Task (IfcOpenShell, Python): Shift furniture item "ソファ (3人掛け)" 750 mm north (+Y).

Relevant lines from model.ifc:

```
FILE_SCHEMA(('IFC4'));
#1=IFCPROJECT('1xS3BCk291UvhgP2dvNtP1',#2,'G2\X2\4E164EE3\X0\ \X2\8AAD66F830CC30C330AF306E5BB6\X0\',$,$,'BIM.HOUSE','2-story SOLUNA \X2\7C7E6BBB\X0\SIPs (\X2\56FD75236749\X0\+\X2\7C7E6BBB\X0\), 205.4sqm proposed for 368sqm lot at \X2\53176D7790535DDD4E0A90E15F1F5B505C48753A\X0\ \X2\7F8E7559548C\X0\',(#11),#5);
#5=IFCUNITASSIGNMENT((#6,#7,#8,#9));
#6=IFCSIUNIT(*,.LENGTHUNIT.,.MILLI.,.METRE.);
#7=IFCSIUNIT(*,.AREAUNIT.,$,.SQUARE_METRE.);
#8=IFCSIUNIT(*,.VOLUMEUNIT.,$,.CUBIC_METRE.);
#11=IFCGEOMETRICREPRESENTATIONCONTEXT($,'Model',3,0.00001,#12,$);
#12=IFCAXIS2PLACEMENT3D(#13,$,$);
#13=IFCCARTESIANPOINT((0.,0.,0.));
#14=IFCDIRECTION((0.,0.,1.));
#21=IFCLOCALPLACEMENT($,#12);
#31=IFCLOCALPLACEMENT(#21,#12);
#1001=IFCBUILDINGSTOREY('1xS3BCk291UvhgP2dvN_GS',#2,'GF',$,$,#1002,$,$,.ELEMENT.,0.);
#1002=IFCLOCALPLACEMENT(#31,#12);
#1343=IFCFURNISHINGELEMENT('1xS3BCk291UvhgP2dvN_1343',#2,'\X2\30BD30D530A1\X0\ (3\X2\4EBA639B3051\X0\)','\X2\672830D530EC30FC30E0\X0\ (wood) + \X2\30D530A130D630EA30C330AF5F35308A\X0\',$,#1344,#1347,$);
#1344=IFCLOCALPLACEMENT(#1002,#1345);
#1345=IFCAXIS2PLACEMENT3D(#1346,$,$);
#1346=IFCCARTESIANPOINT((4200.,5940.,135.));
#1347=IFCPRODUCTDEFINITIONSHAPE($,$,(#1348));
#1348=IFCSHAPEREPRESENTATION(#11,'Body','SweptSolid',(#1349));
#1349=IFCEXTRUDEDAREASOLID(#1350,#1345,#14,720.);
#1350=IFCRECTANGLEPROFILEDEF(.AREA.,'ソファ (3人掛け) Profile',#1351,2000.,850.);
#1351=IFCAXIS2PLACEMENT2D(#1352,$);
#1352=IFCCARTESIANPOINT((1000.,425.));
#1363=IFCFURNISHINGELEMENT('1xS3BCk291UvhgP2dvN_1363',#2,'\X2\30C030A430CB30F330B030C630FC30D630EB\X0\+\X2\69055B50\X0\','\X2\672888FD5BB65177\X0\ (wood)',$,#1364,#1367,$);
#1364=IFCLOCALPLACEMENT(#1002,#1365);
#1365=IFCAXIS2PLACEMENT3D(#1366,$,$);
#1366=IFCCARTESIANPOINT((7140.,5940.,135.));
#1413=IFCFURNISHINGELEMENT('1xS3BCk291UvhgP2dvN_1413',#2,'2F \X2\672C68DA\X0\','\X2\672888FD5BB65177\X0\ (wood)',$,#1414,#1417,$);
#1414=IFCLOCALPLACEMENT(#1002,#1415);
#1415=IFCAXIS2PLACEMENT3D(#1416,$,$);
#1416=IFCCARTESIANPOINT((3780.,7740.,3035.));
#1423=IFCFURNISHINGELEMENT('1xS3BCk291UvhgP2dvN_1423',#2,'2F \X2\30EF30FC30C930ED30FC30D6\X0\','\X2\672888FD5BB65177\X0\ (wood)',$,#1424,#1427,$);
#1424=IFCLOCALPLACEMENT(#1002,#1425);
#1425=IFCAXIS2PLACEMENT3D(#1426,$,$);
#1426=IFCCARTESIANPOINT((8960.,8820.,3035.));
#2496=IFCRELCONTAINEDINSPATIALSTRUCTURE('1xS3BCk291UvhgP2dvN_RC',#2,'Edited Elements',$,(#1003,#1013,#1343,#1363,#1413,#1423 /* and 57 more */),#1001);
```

```python
import ifcopenshell
import ifcopenshell.api.geometry
import ifcopenshell.util.placement

model = ifcopenshell.open("model.ifc")

item = model.by_guid("1xS3BCk291UvhgP2dvN_1343")
matrix = ifcopenshell.util.placement.get_local_placement(item.ObjectPlacement)
matrix[1, 3] += 750.0
ifcopenshell.api.geometry.edit_object_placement(model, product=item, matrix=matrix, is_si=False)

print(ifcopenshell.util.placement.get_local_placement(item.ObjectPlacement).round(3) + 0.0)

model.write("model_rev.ifc")
```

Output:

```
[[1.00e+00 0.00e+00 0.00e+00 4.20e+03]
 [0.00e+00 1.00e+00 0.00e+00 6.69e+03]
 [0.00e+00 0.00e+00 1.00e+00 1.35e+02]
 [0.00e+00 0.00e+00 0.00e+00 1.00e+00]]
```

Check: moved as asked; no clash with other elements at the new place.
